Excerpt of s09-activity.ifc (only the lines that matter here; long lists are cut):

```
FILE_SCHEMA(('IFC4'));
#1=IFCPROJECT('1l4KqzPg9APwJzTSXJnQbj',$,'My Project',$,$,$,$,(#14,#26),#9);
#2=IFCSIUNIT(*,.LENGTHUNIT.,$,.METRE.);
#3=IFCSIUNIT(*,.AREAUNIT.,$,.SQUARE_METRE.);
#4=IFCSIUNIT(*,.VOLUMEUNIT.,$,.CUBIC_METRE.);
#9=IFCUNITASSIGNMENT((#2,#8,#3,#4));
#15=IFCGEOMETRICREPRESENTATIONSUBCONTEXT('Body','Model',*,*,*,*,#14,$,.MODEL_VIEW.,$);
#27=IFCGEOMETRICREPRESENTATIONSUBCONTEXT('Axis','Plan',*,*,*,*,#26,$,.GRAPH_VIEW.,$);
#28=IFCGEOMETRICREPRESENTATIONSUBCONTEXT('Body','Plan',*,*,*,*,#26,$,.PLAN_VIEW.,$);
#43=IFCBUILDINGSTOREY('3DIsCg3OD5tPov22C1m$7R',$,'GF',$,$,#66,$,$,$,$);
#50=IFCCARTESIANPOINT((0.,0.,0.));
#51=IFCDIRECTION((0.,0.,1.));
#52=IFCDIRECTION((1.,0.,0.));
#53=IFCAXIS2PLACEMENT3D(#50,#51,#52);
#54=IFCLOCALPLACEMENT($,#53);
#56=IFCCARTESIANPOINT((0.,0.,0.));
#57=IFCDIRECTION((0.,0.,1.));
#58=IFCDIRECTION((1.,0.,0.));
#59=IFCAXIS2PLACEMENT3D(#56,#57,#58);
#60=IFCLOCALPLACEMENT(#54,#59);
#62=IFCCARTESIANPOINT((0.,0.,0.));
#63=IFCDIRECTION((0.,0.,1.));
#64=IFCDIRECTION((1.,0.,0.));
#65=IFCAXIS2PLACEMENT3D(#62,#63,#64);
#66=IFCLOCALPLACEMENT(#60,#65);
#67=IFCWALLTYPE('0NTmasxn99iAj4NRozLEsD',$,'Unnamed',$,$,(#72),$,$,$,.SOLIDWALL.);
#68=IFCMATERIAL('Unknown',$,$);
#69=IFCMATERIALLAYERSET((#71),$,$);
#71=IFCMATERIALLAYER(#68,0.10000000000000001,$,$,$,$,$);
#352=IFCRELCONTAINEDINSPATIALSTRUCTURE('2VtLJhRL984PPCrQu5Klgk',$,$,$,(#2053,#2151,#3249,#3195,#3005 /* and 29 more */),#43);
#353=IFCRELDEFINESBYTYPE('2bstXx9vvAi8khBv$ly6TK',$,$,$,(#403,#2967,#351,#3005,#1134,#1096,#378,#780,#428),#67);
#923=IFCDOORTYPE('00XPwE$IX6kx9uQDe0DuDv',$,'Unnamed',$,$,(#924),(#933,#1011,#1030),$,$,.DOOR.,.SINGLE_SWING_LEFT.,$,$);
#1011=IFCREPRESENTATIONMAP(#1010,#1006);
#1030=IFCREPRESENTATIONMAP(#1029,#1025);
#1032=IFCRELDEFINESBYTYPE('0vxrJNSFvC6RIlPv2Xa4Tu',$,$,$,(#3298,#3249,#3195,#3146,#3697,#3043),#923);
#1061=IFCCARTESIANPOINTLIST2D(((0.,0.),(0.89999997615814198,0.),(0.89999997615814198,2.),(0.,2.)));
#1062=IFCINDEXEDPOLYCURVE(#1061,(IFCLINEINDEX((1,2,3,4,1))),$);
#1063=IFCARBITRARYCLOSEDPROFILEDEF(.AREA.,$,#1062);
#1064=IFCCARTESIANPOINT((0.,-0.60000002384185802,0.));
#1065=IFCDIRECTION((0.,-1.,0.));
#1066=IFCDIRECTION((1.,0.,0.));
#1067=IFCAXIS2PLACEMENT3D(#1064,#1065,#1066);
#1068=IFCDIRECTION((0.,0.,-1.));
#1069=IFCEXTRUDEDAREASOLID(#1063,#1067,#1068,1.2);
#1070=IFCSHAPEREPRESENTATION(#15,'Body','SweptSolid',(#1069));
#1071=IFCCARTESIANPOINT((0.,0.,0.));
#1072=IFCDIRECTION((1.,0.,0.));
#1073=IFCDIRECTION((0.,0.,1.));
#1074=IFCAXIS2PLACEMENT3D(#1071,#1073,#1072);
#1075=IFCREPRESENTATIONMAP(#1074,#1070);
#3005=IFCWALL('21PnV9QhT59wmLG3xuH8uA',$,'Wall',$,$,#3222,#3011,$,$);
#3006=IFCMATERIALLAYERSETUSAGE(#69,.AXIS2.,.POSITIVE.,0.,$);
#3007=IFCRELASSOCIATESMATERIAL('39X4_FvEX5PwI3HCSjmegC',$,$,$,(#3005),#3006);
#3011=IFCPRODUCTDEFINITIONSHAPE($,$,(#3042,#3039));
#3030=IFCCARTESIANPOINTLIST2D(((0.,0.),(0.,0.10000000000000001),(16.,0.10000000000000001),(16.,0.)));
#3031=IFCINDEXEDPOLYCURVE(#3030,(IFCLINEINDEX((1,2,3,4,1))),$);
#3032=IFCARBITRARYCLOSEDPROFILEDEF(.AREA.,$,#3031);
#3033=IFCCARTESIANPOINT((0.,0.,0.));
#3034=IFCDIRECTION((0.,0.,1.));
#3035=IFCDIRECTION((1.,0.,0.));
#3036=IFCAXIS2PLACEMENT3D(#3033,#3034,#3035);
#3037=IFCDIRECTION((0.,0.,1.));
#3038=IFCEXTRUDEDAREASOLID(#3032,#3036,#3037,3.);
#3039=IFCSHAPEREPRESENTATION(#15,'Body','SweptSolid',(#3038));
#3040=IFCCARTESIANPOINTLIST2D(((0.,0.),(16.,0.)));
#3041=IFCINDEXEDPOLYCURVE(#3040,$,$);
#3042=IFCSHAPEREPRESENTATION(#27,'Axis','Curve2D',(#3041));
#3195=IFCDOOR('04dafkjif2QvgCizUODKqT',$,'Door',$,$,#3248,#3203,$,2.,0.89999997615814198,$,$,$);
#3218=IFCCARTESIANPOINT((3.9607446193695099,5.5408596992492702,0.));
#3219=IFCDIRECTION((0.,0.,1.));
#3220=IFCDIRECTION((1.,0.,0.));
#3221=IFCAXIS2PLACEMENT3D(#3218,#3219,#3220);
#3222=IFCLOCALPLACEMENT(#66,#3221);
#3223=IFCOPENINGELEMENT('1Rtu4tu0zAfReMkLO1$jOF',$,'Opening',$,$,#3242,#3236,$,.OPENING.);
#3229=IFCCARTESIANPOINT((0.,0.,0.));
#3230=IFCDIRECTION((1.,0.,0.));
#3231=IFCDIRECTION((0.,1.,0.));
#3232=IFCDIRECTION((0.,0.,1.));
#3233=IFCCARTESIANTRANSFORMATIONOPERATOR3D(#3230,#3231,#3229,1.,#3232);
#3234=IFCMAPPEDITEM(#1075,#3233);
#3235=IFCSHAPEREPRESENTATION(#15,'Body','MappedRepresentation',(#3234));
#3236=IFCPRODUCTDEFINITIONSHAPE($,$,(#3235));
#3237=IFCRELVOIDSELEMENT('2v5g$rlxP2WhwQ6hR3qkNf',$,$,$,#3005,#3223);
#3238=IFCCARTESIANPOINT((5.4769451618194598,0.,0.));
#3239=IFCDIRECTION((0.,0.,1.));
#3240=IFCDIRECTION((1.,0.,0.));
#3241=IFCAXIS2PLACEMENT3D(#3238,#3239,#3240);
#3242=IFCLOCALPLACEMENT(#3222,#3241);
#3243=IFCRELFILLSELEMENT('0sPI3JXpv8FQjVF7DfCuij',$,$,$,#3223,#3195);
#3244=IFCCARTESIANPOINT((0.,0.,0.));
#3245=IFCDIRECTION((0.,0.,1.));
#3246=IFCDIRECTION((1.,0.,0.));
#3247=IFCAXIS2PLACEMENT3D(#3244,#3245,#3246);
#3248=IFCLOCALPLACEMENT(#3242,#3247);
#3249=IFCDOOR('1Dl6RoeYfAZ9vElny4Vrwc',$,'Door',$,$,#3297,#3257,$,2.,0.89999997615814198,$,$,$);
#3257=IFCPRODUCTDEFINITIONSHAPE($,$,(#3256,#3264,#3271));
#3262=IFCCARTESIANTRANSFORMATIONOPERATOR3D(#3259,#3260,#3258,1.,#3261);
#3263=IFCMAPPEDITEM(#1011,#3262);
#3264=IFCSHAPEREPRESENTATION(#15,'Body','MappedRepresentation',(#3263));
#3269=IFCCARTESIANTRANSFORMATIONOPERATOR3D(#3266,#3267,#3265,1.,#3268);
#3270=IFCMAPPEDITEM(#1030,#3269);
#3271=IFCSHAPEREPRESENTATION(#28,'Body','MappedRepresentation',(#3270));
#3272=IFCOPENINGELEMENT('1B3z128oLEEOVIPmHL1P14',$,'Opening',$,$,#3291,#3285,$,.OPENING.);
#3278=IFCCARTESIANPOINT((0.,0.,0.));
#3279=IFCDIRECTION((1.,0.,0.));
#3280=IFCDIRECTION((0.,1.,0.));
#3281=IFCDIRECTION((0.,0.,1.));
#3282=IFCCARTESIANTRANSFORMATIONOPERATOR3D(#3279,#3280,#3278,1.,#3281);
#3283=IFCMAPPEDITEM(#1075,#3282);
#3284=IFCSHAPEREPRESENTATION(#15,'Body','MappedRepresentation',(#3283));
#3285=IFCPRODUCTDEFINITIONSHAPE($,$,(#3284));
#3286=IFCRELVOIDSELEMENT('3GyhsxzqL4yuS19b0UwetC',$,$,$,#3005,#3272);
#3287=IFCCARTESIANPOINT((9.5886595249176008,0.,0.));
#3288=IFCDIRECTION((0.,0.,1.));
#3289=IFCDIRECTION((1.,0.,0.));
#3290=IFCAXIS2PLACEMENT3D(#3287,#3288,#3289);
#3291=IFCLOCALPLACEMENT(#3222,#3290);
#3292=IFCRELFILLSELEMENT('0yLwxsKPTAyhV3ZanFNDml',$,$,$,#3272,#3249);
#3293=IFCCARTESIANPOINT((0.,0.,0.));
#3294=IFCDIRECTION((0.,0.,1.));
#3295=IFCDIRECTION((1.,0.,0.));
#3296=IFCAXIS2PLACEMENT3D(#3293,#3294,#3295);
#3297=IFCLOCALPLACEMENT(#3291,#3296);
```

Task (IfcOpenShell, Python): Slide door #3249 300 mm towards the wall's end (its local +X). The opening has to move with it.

```python
import ifcopenshell
import ifcopenshell.api.geometry
import ifcopenshell.util.placement
import ifcopenshell.util.unit

model = ifcopenshell.open("s09-activity.ifc")
unit_scale = ifcopenshell.util.unit.calculate_unit_scale(model)

door = model.by_guid("1Dl6RoeYfAZ9vElny4Vrwc")
opening = door.FillsVoids[0].RelatingOpeningElement
wall = opening.VoidsElements[0].RelatingBuildingElement

wall_matrix = ifcopenshell.util.placement.get_local_placement(wall.ObjectPlacement)
shift = wall_matrix[:3, 0] * 0.3 / unit_scale
before = ifcopenshell.util.placement.get_local_placement(door.ObjectPlacement)[:3, 3].copy()

# The door is placed relative to its opening, so it follows when the opening moves.
matrix = ifcopenshell.util.placement.get_local_placement(opening.ObjectPlacement)
matrix[:3, 3] += shift
ifcopenshell.api.geometry.edit_object_placement(
    model, product=opening, matrix=matrix, is_si=False, should_transform_children=True
)

after = ifcopenshell.util.placement.get_local_placement(door.ObjectPlacement)[:3, 3]
print("door moved by", (after - before).round(3) + 0.0)

model.write("s09-activity_v2.ifc")
```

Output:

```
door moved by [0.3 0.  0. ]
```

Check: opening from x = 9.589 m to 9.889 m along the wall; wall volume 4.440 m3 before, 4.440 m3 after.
